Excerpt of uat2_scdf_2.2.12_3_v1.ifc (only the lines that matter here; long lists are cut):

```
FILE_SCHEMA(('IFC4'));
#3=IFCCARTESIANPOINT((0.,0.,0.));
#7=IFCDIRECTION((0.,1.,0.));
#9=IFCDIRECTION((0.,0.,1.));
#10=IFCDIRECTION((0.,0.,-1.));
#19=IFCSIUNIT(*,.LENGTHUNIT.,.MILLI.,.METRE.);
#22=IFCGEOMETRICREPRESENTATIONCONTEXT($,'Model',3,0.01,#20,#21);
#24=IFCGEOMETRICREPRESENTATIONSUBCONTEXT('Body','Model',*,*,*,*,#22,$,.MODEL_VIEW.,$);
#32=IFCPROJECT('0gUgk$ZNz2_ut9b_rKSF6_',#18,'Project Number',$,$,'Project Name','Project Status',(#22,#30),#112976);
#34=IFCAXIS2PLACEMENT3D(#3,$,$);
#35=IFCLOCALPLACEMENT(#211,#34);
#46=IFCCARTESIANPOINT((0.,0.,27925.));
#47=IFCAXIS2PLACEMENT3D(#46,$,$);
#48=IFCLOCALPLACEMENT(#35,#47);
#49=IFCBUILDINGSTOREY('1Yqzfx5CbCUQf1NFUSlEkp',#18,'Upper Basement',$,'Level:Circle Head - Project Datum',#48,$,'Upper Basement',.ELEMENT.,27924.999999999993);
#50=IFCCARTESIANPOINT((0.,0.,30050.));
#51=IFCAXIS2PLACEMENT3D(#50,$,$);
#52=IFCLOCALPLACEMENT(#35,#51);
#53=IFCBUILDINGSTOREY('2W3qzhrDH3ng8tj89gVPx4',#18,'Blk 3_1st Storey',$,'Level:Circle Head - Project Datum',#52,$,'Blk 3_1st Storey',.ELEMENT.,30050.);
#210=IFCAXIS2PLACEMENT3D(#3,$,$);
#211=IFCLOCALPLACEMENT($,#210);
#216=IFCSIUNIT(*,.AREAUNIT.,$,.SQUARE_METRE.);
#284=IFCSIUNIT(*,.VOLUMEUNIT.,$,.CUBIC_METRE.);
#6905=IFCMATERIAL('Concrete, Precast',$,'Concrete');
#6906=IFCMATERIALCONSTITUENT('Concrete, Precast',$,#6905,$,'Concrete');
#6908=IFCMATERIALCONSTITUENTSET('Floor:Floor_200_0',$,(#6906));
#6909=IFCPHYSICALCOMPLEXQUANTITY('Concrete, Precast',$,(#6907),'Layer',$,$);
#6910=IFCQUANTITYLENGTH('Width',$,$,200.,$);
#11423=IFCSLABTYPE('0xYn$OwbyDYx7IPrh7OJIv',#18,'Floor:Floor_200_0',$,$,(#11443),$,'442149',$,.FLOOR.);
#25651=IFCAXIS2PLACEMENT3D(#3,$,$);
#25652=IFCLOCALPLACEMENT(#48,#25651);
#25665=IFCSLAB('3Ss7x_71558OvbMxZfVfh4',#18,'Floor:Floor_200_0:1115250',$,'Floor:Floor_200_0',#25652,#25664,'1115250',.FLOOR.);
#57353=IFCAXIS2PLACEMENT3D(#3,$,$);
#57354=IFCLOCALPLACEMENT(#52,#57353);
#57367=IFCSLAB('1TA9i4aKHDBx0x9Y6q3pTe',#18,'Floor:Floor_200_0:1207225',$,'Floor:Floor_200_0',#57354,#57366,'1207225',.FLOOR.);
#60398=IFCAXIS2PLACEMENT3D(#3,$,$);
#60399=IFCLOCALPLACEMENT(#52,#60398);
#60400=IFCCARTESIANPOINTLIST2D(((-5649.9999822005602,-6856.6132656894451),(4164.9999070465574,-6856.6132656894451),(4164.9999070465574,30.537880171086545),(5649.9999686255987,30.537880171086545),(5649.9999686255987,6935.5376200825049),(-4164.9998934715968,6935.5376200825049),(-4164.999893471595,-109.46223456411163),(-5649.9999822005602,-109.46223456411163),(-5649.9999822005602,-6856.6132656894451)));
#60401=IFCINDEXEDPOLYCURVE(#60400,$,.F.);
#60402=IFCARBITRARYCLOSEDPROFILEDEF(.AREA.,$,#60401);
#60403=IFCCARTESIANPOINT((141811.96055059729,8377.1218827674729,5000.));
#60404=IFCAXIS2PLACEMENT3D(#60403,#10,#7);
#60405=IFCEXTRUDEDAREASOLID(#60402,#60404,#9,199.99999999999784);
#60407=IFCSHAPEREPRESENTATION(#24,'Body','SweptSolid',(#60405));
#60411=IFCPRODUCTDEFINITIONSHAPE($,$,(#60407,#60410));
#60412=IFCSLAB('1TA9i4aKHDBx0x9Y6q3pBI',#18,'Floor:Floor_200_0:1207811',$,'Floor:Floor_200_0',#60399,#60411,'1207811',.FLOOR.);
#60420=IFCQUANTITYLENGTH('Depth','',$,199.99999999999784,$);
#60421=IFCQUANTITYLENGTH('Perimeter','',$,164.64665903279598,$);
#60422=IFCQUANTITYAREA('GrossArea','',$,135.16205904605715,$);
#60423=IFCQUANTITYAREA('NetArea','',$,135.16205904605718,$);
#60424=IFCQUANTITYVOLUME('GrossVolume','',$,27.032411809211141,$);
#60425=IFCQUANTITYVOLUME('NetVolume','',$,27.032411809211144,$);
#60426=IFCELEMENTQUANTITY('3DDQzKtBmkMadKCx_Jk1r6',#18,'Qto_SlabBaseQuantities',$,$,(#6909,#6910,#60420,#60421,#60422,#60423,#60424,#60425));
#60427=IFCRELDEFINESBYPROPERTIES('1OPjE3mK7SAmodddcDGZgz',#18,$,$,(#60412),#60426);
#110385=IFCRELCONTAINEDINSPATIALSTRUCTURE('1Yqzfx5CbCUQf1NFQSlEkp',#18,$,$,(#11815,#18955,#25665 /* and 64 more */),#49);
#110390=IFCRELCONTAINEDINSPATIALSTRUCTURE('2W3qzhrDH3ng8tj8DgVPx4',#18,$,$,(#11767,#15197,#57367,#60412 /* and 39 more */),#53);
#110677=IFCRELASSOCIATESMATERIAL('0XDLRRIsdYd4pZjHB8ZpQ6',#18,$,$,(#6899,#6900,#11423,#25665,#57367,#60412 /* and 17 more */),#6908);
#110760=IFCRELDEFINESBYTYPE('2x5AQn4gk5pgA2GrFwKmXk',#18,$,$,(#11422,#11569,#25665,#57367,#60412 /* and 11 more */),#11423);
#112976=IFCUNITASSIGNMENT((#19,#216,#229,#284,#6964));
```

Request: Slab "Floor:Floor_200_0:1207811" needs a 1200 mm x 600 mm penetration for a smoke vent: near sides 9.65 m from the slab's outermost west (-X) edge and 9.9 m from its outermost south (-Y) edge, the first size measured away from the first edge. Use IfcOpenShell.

```python
import numpy as np
import ifcopenshell
import ifcopenshell.api.feature
import ifcopenshell.api.geometry
import ifcopenshell.api.pset
import ifcopenshell.api.root
import ifcopenshell.geom
import ifcopenshell.util.element
import ifcopenshell.util.placement
import ifcopenshell.util.representation
import ifcopenshell.util.shape
import ifcopenshell.util.unit

model = ifcopenshell.open("uat2_scdf_2.2.12_3_v1.ifc")
unit_scale = ifcopenshell.util.unit.calculate_unit_scale(model)
area_scale = ifcopenshell.util.unit.calculate_unit_scale(model, "AREAUNIT")
volume_scale = ifcopenshell.util.unit.calculate_unit_scale(model, "VOLUMEUNIT")
settings = ifcopenshell.geom.settings()


def volume(element):
    """Net volume in cubic metres, openings subtracted."""
    shape = ifcopenshell.geom.create_shape(settings, element)
    return ifcopenshell.util.shape.get_volume(shape.geometry)


slab = model.by_id(60412)
before = volume(slab)

# Extent in the slab's own axes, in metres. The edges named are its -X and -Y sides.
slab_shape = ifcopenshell.geom.create_shape(settings, slab)
vertices = ifcopenshell.util.shape.get_vertices(slab_shape.geometry)
x_min, y_min, bottom = vertices.min(axis=0)
top = vertices[:, 2].max()

opening = ifcopenshell.api.root.create_entity(model, ifc_class="IfcOpeningElement", name="Smoke vent opening", predefined_type="OPENING")
context = ifcopenshell.util.representation.get_context(model, "Model", "Body", "MODEL_VIEW")
width, depth = 1.2, 0.6
outline = [(0.0, 0.0), (width, 0.0), (width, depth), (0.0, depth), (0.0, 0.0)]
# Overshoot both faces by 50 mm so the cut is clean.
shape = ifcopenshell.api.geometry.add_slab_representation(
    model, context=context, depth=top - bottom + 0.1, polyline=outline
)
ifcopenshell.api.geometry.assign_representation(model, product=opening, representation=shape)

matrix = ifcopenshell.util.placement.get_local_placement(slab.ObjectPlacement)
matrix[:, 3] = matrix @ np.append(np.array([x_min + 9.65, y_min + 9.9, bottom - 0.05]) / unit_scale, 1.0)
ifcopenshell.api.geometry.edit_object_placement(model, product=opening, matrix=matrix, is_si=False)
ifcopenshell.api.feature.add_feature(model, feature=opening, element=slab)

after = volume(slab)

# Update the slab's stored quantities.
qto = model.by_id(ifcopenshell.util.element.get_pset(slab, "Qto_SlabBaseQuantities", should_inherit=False)["id"])
ifcopenshell.api.pset.edit_qto(model, qto=qto, properties={
    "NetArea": after / (top - bottom) / area_scale,
    "NetVolume": after / volume_scale,
})

print(f"slab volume {before:.3f} -> {after:.3f} m3")

model.write("uat2_scdf_2.2.12_3_v1_v2.ifc")
```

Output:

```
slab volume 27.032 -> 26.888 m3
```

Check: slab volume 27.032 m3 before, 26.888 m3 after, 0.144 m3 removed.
